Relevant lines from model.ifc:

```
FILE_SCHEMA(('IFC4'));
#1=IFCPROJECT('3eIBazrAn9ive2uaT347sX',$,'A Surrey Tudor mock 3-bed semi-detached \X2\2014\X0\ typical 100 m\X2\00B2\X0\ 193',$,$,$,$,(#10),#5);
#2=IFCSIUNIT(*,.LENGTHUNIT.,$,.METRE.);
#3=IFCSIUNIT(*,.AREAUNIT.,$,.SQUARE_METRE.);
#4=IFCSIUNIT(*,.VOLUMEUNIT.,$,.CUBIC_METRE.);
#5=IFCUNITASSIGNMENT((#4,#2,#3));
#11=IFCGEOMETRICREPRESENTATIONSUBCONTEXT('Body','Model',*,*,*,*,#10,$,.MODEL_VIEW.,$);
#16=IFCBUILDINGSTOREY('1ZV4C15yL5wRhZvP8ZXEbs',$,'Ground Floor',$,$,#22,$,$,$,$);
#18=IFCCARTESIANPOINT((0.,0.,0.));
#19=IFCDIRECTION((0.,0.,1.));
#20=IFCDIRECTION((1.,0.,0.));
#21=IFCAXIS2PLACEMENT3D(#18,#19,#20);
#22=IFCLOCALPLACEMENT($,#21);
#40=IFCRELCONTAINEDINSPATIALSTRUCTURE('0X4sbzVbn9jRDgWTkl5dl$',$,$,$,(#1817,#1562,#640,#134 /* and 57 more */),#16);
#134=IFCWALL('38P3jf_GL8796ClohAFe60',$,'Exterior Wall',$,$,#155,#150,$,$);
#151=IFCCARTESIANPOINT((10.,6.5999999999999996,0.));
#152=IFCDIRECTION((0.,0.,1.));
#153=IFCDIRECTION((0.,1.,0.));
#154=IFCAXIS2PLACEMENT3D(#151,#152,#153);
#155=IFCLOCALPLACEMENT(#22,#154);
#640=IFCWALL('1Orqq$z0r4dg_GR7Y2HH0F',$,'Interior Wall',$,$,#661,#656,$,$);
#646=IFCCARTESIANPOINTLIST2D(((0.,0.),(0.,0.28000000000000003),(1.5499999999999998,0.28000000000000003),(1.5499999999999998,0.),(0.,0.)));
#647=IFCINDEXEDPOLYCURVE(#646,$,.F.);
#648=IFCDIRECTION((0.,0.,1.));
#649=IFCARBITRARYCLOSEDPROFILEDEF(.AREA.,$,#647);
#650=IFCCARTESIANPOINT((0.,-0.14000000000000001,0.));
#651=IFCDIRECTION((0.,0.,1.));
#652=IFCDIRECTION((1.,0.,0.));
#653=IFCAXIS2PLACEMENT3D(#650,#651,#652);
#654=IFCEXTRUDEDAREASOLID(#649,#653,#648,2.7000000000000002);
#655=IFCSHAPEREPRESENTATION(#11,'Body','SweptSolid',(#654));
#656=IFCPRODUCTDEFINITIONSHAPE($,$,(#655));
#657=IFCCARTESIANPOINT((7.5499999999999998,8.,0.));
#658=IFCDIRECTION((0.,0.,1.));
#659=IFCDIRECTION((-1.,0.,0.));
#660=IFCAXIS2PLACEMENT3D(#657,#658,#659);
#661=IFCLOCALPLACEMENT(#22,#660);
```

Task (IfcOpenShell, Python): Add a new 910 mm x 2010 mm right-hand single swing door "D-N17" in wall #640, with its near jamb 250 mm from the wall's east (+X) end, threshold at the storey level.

```python
import numpy as np
import ifcopenshell
import ifcopenshell.api.feature
import ifcopenshell.api.geometry
import ifcopenshell.api.root
import ifcopenshell.api.spatial
import ifcopenshell.geom
import ifcopenshell.util.element
import ifcopenshell.util.placement
import ifcopenshell.util.representation
import ifcopenshell.util.shape
import ifcopenshell.util.unit

model = ifcopenshell.open("model.ifc")
unit_scale = ifcopenshell.util.unit.calculate_unit_scale(model)
settings = ifcopenshell.geom.settings()


def volume(element):
    """Net volume in cubic metres, openings subtracted."""
    shape = ifcopenshell.geom.create_shape(settings, element)
    return ifcopenshell.util.shape.get_volume(shape.geometry)


wall = model.by_guid("1Orqq$z0r4dg_GR7Y2HH0F")
storey = ifcopenshell.util.element.get_container(wall, ifc_class="IfcBuildingStorey")
context = ifcopenshell.util.representation.get_context(model, "Model", "Body", "MODEL_VIEW")
before = volume(wall)

width, height, from_end, sill = 0.91, 2.01, 0.25, 0.0  # metres

# The wall runs along its own X axis, and the end named is its -X end.
wall_shape = ifcopenshell.geom.create_shape(settings, wall)
x, y, z = ifcopenshell.util.shape.get_vertices(wall_shape.geometry).T
start = x.min() + from_end
face, thickness = float(y.min()), float(y.max() - y.min())
wall_matrix = ifcopenshell.util.placement.get_local_placement(wall.ObjectPlacement)
level = ifcopenshell.util.placement.get_local_placement(storey.ObjectPlacement)[2, 3]


def in_wall(x, y):
    """Placement at x, y metres in the wall's axes, at sill height."""
    matrix = wall_matrix.copy()
    matrix[:, 3] = wall_matrix @ np.array([x / unit_scale, y / unit_scale, 0.0, 1.0])
    matrix[2, 3] = level + sill / unit_scale
    return matrix


# Opening: a box that overshoots both wall faces by 50 mm.
opening = ifcopenshell.api.root.create_entity(model, ifc_class="IfcOpeningElement", predefined_type="OPENING")
box = ifcopenshell.api.geometry.add_wall_representation(
    model, context=context, length=width, height=height, thickness=thickness + 0.1
)
ifcopenshell.api.geometry.assign_representation(model, product=opening, representation=box)
ifcopenshell.api.geometry.edit_object_placement(model, product=opening, matrix=in_wall(start, face - 0.05), is_si=False)
ifcopenshell.api.feature.add_feature(model, feature=opening, element=wall)

door = ifcopenshell.api.root.create_entity(model, ifc_class="IfcDoor", name="D-N17", predefined_type="DOOR")
door.OverallWidth, door.OverallHeight = width / unit_scale, height / unit_scale
door.OperationType = "SINGLE_SWING_RIGHT"
body = ifcopenshell.api.geometry.add_door_representation(
    model,
    context=context,
    overall_width=door.OverallWidth,
    overall_height=door.OverallHeight,
    operation_type="SINGLE_SWING_RIGHT",
    lining_properties={"LiningDepth": thickness / unit_scale, "ThresholdDepth": thickness / unit_scale},
)
ifcopenshell.api.geometry.assign_representation(model, product=door, representation=body)
ifcopenshell.api.spatial.assign_container(model, products=[door], relating_structure=storey)
ifcopenshell.api.feature.add_filling(model, opening=opening, element=door)

# The lining spans the wall, so the door starts at the wall face.
ifcopenshell.api.geometry.edit_object_placement(model, product=door, matrix=in_wall(start, face), is_si=False)

after = volume(wall)

print(f"wall volume {before:.3f} -> {after:.3f} m3")

model.write("model_updated.ifc")
```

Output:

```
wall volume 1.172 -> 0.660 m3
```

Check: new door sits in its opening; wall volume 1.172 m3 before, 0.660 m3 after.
